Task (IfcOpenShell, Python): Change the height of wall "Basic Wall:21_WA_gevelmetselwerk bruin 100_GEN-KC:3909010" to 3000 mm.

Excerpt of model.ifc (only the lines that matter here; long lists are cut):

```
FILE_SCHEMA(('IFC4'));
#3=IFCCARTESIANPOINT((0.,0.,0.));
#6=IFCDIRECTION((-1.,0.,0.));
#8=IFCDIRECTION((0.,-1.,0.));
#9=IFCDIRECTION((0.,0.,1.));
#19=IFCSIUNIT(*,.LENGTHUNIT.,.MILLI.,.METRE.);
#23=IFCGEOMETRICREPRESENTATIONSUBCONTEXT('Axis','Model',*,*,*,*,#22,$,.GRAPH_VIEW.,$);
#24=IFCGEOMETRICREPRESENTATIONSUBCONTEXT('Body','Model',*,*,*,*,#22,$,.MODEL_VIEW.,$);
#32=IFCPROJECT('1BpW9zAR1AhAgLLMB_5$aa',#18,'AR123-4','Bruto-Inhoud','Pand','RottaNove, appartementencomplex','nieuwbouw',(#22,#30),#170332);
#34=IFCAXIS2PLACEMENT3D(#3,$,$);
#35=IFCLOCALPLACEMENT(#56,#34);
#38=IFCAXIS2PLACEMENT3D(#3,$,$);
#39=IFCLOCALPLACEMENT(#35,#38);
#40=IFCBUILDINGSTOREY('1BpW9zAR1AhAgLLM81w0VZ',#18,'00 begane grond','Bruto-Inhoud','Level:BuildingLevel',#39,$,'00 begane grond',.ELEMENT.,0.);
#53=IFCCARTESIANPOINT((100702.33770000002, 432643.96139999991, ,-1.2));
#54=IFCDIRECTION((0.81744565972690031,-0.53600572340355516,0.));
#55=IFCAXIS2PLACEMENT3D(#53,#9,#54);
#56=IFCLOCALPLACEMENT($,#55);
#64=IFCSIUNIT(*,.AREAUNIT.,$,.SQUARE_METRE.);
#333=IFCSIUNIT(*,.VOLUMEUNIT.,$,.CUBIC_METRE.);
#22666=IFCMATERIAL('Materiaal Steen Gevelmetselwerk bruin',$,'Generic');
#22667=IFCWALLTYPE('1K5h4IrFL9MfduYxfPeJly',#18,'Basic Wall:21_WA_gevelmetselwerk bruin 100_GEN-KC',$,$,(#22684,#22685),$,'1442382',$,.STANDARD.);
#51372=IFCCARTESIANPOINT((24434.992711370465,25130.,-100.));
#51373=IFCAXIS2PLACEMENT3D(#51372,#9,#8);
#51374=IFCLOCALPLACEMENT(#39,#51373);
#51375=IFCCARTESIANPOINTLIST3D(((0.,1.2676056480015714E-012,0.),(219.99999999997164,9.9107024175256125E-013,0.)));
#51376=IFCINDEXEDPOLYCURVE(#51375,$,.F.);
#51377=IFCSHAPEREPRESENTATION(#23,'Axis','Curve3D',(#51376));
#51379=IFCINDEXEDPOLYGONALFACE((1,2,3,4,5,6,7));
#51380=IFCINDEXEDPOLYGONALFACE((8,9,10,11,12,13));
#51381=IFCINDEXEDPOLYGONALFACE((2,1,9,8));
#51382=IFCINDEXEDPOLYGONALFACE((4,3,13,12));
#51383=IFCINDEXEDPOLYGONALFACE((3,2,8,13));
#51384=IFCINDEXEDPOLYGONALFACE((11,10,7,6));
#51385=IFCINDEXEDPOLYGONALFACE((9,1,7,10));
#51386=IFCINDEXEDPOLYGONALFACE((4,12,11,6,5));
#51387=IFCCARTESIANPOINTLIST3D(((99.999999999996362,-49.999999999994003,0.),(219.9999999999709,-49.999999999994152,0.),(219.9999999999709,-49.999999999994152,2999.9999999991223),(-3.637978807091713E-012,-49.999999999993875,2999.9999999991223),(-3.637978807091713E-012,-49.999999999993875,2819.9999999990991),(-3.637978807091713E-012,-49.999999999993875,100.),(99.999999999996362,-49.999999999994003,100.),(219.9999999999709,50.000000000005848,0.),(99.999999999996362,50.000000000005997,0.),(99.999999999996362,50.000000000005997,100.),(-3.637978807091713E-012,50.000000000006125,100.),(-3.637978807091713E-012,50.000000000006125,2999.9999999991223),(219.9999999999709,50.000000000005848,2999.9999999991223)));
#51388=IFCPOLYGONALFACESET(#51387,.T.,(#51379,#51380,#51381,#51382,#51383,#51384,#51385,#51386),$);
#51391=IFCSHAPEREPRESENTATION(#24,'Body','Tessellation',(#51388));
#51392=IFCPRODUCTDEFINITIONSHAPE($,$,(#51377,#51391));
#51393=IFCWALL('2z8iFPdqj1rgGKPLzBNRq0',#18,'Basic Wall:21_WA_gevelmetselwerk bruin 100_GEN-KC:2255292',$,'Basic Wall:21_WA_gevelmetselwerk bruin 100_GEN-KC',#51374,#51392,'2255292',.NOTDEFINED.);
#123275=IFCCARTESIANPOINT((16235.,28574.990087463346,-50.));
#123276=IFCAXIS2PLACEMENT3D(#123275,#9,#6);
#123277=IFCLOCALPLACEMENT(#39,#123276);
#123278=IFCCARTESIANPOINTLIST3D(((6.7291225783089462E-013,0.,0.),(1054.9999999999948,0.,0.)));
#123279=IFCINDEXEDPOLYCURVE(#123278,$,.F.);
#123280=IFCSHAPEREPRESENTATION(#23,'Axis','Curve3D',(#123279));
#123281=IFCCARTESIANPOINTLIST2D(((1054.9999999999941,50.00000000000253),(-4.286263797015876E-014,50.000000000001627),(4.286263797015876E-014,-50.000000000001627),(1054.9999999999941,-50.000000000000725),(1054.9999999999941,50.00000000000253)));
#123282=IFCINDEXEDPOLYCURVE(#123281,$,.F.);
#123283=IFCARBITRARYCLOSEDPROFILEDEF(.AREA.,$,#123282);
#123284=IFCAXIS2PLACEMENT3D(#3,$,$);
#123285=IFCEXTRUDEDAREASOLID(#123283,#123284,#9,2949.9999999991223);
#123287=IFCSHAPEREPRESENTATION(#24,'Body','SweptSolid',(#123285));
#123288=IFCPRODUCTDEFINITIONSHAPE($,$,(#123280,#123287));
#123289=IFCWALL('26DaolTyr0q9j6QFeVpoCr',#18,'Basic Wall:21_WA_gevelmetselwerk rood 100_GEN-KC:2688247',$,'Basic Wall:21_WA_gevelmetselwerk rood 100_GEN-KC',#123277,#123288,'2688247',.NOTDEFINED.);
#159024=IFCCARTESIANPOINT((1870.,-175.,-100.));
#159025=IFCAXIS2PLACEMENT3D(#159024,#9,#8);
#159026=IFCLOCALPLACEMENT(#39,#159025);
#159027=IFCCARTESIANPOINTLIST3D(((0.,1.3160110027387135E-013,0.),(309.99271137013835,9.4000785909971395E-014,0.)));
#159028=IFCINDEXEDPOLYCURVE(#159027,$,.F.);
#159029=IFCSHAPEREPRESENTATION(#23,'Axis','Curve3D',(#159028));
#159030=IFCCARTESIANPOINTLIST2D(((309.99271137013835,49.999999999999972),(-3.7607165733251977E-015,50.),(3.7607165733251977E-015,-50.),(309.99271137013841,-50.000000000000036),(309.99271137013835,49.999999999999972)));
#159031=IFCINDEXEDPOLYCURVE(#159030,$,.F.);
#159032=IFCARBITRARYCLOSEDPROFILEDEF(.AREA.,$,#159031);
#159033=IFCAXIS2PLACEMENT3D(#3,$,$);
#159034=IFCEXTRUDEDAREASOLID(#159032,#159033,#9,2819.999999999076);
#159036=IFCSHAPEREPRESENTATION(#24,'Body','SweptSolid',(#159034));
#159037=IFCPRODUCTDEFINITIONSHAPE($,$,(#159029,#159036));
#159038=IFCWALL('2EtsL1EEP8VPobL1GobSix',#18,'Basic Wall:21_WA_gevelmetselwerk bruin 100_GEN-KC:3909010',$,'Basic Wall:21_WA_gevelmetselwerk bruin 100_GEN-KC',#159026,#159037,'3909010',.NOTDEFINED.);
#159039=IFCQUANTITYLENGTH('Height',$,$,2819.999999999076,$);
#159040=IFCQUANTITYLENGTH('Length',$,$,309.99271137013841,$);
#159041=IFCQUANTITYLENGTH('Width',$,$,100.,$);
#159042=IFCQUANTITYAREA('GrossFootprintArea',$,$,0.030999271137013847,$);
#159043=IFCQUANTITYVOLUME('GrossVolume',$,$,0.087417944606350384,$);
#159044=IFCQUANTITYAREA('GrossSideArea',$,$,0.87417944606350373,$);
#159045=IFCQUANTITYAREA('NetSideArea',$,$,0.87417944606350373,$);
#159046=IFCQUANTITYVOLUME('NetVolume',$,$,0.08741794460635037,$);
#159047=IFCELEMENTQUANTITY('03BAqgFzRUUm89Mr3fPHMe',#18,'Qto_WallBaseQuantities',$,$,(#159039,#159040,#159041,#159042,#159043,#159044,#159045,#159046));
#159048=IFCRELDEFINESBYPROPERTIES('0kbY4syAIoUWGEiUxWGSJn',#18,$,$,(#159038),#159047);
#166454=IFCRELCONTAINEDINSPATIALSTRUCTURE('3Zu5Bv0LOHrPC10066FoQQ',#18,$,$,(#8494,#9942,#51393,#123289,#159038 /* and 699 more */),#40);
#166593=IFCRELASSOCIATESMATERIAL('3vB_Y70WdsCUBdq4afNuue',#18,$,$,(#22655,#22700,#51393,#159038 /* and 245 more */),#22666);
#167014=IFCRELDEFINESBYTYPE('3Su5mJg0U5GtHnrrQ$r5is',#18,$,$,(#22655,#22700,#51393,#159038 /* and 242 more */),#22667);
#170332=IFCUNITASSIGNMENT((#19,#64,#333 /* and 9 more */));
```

```python
import ifcopenshell
import ifcopenshell.api.pset
import ifcopenshell.geom
import ifcopenshell.util.element
import ifcopenshell.util.representation
import ifcopenshell.util.shape
import ifcopenshell.util.unit

model = ifcopenshell.open("model.ifc")
unit_scale = ifcopenshell.util.unit.calculate_unit_scale(model)
area_scale = ifcopenshell.util.unit.calculate_unit_scale(model, "AREAUNIT")
volume_scale = ifcopenshell.util.unit.calculate_unit_scale(model, "VOLUMEUNIT")
settings = ifcopenshell.geom.settings()


def volume(element):
    """Net volume in cubic metres, openings subtracted."""
    shape = ifcopenshell.geom.create_shape(settings, element)
    return ifcopenshell.util.shape.get_volume(shape.geometry)


wall = model.by_id(159038)
before = volume(wall)

body = ifcopenshell.util.representation.get_representation(wall, "Model", "Body")
solid = body.Items[0]
old_height = solid.Depth
solid.Depth = 3 / unit_scale
after = volume(wall)
thickness = 0.1  # wall thickness in metres

# Update the stored height, areas and volumes.
qto = model.by_id(ifcopenshell.util.element.get_pset(wall, "Qto_WallBaseQuantities", should_inherit=False)["id"])
ifcopenshell.api.pset.edit_qto(model, qto=qto, properties={
    "Height": solid.Depth,
    "GrossVolume": ifcopenshell.util.element.get_pset(wall, "Qto_WallBaseQuantities", "GrossVolume") * solid.Depth / old_height,
    "GrossSideArea": ifcopenshell.util.element.get_pset(wall, "Qto_WallBaseQuantities", "GrossSideArea") * solid.Depth / old_height,
    "NetSideArea": after / thickness / area_scale,
    "NetVolume": after / volume_scale,
})

print(f"height {old_height:g} -> {solid.Depth:g}, volume {before:.3f} -> {after:.3f} m3")

model.write("model_v2.ifc")
```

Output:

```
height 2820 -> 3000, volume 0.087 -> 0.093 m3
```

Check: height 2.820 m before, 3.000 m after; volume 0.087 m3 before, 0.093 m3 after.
